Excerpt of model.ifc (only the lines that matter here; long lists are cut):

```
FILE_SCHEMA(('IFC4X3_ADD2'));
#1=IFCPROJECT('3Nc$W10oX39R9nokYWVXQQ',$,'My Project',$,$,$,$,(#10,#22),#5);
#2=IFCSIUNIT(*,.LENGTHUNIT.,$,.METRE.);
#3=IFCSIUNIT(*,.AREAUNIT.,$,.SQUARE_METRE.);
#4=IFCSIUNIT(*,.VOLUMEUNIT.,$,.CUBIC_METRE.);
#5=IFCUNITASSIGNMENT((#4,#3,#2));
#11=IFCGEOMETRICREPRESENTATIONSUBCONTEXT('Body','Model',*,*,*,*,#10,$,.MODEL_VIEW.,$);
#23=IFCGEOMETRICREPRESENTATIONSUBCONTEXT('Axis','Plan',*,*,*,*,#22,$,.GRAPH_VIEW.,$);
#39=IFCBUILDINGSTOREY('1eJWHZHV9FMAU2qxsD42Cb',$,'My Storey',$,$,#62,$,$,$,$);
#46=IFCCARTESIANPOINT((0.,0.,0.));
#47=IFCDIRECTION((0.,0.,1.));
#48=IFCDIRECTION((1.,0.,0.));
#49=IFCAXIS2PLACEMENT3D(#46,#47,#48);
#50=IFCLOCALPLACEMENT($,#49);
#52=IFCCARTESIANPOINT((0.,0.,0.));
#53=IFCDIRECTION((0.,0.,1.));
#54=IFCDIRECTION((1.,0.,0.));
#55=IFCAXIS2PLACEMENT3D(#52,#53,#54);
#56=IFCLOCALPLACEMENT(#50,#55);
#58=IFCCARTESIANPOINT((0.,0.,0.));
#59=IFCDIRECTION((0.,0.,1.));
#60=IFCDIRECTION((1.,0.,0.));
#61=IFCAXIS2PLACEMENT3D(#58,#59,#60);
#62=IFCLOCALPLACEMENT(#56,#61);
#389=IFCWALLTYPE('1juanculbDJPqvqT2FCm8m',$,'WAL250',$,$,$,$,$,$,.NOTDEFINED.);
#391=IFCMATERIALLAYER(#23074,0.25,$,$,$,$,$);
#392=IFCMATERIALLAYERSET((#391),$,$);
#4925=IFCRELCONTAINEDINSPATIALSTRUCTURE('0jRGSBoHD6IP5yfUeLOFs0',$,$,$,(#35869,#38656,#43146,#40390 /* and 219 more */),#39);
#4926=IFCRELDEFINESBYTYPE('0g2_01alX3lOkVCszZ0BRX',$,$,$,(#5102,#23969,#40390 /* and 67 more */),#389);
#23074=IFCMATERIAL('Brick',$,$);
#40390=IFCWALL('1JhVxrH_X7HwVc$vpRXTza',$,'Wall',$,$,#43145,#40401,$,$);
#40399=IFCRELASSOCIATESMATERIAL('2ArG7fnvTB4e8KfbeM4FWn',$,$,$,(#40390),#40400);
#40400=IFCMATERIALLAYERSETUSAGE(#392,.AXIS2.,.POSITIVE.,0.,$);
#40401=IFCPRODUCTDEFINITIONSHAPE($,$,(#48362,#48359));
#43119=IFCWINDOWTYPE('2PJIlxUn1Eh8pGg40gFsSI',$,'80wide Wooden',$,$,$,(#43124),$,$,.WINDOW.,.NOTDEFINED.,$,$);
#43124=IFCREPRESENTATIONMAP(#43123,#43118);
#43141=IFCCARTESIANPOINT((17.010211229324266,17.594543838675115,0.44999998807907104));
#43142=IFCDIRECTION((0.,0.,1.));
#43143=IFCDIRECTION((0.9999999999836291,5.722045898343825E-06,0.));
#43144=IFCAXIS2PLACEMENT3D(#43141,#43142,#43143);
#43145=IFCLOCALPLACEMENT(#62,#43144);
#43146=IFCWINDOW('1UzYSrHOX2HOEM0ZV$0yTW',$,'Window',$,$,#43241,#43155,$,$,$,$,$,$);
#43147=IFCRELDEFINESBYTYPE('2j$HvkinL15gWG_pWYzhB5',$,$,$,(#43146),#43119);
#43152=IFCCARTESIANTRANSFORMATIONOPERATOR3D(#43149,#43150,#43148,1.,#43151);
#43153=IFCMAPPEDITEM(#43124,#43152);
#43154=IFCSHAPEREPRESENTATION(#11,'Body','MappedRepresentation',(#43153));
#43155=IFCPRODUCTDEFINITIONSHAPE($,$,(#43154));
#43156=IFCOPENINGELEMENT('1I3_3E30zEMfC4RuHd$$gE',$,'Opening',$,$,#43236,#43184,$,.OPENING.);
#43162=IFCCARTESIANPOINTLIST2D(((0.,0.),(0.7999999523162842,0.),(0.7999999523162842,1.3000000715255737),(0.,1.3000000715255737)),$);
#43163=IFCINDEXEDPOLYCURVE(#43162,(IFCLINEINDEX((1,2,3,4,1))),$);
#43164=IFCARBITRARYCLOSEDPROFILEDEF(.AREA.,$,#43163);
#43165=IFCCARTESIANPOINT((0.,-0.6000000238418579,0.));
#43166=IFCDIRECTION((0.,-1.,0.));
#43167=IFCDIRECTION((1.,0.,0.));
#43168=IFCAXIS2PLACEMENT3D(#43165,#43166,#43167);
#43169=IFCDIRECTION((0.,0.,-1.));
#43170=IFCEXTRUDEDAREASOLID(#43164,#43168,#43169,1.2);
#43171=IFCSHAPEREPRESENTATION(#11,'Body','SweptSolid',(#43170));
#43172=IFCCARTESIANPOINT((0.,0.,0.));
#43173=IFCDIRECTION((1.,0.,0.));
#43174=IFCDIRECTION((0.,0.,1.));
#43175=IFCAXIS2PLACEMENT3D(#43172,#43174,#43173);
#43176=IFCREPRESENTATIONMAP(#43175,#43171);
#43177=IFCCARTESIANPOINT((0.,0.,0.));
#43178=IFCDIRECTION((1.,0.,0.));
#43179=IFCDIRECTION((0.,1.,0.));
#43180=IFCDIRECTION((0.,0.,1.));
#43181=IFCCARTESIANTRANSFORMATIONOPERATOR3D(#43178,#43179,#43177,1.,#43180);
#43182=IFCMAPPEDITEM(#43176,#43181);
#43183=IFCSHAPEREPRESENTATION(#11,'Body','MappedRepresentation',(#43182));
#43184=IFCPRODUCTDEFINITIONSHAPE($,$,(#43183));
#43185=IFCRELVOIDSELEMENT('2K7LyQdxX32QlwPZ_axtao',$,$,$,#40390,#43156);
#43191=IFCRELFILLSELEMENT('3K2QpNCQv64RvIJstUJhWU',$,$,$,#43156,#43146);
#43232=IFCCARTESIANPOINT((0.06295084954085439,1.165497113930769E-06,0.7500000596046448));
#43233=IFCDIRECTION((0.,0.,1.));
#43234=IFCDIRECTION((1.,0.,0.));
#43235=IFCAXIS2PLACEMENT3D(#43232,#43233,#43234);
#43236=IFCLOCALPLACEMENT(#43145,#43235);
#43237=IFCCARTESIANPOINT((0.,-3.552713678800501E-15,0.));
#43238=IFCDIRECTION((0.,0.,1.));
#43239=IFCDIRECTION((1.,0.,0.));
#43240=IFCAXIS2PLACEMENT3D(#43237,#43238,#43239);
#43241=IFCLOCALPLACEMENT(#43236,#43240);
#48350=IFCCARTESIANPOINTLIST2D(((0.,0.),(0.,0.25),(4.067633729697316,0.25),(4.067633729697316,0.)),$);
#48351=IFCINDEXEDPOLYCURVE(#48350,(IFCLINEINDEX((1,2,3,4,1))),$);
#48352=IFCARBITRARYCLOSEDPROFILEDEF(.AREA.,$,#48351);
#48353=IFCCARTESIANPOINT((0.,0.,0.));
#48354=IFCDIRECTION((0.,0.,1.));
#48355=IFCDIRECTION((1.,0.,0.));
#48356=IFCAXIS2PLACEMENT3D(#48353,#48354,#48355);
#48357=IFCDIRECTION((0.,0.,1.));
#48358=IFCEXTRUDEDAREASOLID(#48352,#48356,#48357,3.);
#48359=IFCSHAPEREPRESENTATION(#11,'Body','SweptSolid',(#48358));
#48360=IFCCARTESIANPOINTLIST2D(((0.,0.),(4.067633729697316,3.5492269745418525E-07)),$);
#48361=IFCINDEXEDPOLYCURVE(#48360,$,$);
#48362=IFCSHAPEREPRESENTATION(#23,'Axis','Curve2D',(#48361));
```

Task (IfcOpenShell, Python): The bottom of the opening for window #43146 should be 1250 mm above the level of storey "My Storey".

```python
import numpy as np
import ifcopenshell
import ifcopenshell.api.geometry
import ifcopenshell.geom
import ifcopenshell.util.element
import ifcopenshell.util.placement
import ifcopenshell.util.shape
import ifcopenshell.util.unit

model = ifcopenshell.open("model.ifc")
unit_scale = ifcopenshell.util.unit.calculate_unit_scale(model)

window = model.by_guid("1UzYSrHOX2HOEM0ZV$0yTW")
opening = window.FillsVoids[0].RelatingOpeningElement
storey = ifcopenshell.util.element.get_container(window, ifc_class="IfcBuildingStorey")
level = ifcopenshell.util.placement.get_local_placement(storey.ObjectPlacement)[2, 3]

# The opening's origin need not be at the sill, so measure its lowest point.
shape = ifcopenshell.geom.create_shape(ifcopenshell.geom.settings(), opening)
bottom = ifcopenshell.util.shape.get_shape_bottom_elevation(shape, shape.geometry) / unit_scale
dz = level + 1.25 - bottom

shift = np.array([0.0, 0.0, dz])
# The window is placed relative to its opening, so it follows when the opening moves.
matrix = ifcopenshell.util.placement.get_local_placement(opening.ObjectPlacement)
matrix[:3, 3] += shift
ifcopenshell.api.geometry.edit_object_placement(
    model, product=opening, matrix=matrix, is_si=False, should_transform_children=True
)

print(f"moved by {dz * unit_scale:+.3f} m")

model.write("model-out.ifc")
```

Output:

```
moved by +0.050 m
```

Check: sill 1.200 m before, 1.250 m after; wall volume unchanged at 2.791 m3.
